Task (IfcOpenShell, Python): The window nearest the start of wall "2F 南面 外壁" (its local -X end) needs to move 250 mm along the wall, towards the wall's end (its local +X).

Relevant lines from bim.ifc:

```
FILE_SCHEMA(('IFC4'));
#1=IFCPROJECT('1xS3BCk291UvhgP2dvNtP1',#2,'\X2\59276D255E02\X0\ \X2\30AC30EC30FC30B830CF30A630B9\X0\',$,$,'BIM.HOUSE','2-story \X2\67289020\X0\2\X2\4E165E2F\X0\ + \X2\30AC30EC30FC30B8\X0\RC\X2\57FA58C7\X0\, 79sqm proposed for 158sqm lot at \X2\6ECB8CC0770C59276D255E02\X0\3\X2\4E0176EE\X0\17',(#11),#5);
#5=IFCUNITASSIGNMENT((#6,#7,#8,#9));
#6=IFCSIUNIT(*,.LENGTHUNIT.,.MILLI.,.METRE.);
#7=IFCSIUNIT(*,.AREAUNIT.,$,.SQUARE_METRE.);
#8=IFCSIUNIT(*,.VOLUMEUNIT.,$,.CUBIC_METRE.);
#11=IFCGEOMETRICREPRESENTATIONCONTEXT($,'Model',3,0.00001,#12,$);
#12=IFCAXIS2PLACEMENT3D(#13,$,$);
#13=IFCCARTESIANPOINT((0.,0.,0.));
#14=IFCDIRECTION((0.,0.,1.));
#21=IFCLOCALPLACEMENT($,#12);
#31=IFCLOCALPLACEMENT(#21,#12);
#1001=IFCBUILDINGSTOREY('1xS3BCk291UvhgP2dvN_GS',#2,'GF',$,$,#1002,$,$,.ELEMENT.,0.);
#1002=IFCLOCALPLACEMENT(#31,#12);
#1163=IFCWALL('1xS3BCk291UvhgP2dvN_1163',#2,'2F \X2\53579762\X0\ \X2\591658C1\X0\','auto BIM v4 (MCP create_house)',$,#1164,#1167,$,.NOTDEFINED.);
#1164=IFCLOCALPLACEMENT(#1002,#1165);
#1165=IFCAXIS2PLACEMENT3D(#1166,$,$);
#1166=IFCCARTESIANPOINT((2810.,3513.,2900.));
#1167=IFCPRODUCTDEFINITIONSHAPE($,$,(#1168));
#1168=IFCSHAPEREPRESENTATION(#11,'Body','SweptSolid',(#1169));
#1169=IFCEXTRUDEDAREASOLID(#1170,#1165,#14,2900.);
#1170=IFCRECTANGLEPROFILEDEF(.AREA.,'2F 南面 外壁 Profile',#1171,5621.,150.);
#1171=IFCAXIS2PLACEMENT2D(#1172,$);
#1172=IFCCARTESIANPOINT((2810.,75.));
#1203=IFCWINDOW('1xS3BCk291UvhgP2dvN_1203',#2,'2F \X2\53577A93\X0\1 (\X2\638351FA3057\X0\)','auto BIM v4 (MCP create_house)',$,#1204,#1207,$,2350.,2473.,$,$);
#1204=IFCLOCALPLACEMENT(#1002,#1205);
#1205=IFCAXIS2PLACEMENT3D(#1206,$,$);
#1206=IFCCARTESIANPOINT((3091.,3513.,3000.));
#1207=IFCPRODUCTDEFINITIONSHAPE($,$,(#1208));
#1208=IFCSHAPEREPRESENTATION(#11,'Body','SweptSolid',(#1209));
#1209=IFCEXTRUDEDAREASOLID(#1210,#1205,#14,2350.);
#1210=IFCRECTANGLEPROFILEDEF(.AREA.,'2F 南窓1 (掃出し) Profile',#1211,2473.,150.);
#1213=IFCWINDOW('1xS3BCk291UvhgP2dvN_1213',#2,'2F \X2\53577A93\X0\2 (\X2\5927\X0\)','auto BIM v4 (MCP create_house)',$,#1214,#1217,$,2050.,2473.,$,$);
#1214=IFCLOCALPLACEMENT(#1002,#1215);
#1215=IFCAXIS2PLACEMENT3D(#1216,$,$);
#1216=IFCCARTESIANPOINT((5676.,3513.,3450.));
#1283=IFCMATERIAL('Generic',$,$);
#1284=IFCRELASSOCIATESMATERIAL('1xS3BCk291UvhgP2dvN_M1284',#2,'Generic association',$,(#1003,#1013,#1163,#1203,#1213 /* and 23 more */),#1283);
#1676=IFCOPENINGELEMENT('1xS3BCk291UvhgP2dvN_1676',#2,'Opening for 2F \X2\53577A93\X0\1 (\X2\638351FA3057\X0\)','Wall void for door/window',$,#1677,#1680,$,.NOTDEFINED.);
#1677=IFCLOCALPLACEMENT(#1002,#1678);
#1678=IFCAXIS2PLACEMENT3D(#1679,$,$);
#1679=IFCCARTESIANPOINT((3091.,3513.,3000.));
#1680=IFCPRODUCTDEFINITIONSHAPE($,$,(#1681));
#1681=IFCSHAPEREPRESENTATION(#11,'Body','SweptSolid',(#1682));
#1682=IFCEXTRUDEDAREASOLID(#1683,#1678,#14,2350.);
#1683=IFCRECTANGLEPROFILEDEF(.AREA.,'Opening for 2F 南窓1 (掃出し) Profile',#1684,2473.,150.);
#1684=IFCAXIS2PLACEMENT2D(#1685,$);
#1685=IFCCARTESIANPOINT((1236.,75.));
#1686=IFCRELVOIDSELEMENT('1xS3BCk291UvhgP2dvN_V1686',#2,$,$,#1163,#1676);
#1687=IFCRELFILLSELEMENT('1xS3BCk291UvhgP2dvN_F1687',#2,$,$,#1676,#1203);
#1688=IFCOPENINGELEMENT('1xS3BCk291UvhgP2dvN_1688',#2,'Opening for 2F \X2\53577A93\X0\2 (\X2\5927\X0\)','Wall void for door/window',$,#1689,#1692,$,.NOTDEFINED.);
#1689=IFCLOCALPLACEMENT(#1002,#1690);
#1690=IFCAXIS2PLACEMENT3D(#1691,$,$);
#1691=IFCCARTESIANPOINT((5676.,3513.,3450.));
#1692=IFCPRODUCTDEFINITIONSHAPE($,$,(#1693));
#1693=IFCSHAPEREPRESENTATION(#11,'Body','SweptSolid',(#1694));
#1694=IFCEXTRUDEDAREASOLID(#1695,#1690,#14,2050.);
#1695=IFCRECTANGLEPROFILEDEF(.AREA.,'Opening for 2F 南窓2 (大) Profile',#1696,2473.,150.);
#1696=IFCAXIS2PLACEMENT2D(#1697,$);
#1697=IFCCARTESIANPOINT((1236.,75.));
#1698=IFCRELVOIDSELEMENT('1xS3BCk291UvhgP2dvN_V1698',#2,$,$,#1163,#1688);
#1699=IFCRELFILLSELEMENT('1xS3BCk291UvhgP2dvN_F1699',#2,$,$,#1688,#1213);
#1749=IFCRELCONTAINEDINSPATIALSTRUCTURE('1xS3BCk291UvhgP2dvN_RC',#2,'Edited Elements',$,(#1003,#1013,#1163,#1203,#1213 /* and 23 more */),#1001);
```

```python
import ifcopenshell
import ifcopenshell.api.geometry
import ifcopenshell.util.placement
import ifcopenshell.util.unit

model = ifcopenshell.open("bim.ifc")
unit_scale = ifcopenshell.util.unit.calculate_unit_scale(model)

window = model.by_guid("1xS3BCk291UvhgP2dvN_1203")
opening = window.FillsVoids[0].RelatingOpeningElement
wall = opening.VoidsElements[0].RelatingBuildingElement

wall_matrix = ifcopenshell.util.placement.get_local_placement(wall.ObjectPlacement)
shift = wall_matrix[:3, 0] * 0.25 / unit_scale
before = ifcopenshell.util.placement.get_local_placement(window.ObjectPlacement)[:3, 3].copy()

# The window is not placed relative to its opening, so move both.
for product in (opening, window):
    matrix = ifcopenshell.util.placement.get_local_placement(product.ObjectPlacement)
    matrix[:3, 3] += shift
    ifcopenshell.api.geometry.edit_object_placement(model, product=product, matrix=matrix, is_si=False)

after = ifcopenshell.util.placement.get_local_placement(window.ObjectPlacement)[:3, 3]
print("window moved by", (after - before).round(3) + 0.0)

model.write("bim_edited.ifc")
```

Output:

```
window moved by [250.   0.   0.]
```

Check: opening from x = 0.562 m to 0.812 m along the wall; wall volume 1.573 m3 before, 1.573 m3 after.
